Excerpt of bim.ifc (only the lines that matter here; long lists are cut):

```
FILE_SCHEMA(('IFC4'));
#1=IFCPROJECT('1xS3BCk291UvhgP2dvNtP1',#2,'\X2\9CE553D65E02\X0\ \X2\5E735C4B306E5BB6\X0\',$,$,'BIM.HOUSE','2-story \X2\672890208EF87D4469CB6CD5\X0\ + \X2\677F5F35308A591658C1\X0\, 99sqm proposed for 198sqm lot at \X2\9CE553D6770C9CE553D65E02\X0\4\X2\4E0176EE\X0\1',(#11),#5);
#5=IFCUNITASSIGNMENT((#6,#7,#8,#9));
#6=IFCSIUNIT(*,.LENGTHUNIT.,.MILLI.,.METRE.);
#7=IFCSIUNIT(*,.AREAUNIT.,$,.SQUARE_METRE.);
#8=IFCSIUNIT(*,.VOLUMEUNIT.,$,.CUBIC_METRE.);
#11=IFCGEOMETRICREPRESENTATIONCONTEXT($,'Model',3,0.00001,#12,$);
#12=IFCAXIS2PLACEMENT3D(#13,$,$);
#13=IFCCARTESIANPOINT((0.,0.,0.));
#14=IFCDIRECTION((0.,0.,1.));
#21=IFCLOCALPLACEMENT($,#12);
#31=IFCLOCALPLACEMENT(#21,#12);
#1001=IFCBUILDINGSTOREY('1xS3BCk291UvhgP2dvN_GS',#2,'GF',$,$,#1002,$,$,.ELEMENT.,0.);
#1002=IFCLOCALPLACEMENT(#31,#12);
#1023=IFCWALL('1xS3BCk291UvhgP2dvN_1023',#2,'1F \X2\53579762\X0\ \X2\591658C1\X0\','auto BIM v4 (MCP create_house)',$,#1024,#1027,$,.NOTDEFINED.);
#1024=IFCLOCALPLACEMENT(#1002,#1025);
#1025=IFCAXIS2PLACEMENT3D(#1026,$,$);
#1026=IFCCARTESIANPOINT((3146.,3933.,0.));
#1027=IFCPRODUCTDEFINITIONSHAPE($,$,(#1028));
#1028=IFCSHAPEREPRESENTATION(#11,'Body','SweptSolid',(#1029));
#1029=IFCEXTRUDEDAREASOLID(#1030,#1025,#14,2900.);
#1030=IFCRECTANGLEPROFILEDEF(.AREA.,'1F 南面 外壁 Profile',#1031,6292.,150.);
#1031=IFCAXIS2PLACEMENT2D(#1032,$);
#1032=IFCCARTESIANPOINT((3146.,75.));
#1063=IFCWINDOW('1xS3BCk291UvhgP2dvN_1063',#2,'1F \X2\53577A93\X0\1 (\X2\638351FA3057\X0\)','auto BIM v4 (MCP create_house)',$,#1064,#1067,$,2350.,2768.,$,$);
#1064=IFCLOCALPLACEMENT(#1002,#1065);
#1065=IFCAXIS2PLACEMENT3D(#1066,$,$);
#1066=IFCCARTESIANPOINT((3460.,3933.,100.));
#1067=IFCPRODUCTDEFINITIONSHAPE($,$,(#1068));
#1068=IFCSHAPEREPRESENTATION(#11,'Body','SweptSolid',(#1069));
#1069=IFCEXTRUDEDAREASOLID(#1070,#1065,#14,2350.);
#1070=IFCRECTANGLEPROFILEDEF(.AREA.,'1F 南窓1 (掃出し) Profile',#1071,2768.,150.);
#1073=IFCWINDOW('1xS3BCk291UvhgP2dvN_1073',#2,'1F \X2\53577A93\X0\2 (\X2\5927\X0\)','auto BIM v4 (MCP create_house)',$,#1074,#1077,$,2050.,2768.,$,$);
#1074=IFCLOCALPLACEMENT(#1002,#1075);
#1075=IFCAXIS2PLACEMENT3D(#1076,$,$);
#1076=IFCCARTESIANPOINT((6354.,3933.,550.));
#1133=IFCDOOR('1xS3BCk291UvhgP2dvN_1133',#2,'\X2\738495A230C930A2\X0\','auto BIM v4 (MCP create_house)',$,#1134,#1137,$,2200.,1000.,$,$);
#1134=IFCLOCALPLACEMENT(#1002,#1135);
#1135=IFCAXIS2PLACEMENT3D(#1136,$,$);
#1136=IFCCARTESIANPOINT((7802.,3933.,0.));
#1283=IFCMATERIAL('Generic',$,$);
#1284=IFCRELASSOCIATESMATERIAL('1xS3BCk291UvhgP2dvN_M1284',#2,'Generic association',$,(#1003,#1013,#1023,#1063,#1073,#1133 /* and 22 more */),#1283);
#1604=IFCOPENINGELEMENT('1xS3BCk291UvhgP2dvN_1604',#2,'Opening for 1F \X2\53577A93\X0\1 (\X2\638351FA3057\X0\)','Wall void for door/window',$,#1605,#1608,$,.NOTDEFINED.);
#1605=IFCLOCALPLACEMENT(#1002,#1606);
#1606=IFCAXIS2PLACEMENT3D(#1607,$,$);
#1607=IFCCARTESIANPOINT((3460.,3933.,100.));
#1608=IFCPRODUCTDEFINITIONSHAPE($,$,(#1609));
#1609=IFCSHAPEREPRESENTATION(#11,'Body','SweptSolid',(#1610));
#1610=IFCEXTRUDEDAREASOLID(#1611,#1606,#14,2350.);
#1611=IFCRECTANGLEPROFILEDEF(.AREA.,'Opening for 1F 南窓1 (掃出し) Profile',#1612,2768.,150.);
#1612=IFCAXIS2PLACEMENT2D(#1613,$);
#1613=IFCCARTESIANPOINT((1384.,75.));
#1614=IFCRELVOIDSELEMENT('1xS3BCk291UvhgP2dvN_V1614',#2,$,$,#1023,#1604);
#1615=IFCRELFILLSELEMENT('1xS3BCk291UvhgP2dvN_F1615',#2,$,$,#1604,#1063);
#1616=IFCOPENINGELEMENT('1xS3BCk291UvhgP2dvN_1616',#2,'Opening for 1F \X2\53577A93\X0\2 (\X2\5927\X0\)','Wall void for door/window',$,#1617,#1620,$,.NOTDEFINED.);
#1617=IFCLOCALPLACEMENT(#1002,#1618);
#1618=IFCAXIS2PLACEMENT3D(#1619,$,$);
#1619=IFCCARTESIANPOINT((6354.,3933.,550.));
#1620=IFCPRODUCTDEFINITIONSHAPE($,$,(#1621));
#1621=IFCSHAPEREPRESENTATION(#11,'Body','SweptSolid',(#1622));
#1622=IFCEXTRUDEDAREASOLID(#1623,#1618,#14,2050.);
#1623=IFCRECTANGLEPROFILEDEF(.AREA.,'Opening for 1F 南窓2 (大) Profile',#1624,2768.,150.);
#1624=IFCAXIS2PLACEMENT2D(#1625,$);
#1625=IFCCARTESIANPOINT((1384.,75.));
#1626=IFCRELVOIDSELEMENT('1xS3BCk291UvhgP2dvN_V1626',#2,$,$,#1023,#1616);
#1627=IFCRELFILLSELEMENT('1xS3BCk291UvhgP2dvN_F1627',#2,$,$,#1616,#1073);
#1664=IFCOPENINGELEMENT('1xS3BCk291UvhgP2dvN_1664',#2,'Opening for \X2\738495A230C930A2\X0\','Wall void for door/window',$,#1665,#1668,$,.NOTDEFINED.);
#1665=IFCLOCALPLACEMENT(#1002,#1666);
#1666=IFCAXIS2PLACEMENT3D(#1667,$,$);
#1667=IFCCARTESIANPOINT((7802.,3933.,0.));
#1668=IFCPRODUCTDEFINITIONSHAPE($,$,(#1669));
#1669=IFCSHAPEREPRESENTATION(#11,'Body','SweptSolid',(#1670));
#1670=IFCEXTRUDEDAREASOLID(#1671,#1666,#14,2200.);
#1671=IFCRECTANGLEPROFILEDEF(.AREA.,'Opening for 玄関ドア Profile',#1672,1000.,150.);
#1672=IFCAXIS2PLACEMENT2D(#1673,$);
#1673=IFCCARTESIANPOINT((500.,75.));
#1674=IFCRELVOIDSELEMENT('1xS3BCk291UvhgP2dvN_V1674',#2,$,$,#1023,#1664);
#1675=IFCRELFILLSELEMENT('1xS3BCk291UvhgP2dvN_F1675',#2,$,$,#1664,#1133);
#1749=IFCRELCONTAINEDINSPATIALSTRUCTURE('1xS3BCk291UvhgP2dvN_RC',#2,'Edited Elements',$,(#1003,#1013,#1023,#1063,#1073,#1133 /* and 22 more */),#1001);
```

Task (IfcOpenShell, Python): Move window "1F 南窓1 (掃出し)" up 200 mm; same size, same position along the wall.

```python
import numpy as np
import ifcopenshell
import ifcopenshell.api.geometry
import ifcopenshell.util.placement
import ifcopenshell.util.unit

model = ifcopenshell.open("bim.ifc")
unit_scale = ifcopenshell.util.unit.calculate_unit_scale(model)

window = model.by_guid("1xS3BCk291UvhgP2dvN_1063")
opening = window.FillsVoids[0].RelatingOpeningElement
dz = 200.0

shift = np.array([0.0, 0.0, dz])
# The window is not placed relative to its opening, so move both.
for product in (opening, window):
    matrix = ifcopenshell.util.placement.get_local_placement(product.ObjectPlacement)
    matrix[:3, 3] += shift
    ifcopenshell.api.geometry.edit_object_placement(model, product=product, matrix=matrix, is_si=False)

print(f"moved by {dz * unit_scale:+.3f} m")

model.write("bim_v2.ifc")
```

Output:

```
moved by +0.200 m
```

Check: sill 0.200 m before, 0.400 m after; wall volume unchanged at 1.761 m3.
